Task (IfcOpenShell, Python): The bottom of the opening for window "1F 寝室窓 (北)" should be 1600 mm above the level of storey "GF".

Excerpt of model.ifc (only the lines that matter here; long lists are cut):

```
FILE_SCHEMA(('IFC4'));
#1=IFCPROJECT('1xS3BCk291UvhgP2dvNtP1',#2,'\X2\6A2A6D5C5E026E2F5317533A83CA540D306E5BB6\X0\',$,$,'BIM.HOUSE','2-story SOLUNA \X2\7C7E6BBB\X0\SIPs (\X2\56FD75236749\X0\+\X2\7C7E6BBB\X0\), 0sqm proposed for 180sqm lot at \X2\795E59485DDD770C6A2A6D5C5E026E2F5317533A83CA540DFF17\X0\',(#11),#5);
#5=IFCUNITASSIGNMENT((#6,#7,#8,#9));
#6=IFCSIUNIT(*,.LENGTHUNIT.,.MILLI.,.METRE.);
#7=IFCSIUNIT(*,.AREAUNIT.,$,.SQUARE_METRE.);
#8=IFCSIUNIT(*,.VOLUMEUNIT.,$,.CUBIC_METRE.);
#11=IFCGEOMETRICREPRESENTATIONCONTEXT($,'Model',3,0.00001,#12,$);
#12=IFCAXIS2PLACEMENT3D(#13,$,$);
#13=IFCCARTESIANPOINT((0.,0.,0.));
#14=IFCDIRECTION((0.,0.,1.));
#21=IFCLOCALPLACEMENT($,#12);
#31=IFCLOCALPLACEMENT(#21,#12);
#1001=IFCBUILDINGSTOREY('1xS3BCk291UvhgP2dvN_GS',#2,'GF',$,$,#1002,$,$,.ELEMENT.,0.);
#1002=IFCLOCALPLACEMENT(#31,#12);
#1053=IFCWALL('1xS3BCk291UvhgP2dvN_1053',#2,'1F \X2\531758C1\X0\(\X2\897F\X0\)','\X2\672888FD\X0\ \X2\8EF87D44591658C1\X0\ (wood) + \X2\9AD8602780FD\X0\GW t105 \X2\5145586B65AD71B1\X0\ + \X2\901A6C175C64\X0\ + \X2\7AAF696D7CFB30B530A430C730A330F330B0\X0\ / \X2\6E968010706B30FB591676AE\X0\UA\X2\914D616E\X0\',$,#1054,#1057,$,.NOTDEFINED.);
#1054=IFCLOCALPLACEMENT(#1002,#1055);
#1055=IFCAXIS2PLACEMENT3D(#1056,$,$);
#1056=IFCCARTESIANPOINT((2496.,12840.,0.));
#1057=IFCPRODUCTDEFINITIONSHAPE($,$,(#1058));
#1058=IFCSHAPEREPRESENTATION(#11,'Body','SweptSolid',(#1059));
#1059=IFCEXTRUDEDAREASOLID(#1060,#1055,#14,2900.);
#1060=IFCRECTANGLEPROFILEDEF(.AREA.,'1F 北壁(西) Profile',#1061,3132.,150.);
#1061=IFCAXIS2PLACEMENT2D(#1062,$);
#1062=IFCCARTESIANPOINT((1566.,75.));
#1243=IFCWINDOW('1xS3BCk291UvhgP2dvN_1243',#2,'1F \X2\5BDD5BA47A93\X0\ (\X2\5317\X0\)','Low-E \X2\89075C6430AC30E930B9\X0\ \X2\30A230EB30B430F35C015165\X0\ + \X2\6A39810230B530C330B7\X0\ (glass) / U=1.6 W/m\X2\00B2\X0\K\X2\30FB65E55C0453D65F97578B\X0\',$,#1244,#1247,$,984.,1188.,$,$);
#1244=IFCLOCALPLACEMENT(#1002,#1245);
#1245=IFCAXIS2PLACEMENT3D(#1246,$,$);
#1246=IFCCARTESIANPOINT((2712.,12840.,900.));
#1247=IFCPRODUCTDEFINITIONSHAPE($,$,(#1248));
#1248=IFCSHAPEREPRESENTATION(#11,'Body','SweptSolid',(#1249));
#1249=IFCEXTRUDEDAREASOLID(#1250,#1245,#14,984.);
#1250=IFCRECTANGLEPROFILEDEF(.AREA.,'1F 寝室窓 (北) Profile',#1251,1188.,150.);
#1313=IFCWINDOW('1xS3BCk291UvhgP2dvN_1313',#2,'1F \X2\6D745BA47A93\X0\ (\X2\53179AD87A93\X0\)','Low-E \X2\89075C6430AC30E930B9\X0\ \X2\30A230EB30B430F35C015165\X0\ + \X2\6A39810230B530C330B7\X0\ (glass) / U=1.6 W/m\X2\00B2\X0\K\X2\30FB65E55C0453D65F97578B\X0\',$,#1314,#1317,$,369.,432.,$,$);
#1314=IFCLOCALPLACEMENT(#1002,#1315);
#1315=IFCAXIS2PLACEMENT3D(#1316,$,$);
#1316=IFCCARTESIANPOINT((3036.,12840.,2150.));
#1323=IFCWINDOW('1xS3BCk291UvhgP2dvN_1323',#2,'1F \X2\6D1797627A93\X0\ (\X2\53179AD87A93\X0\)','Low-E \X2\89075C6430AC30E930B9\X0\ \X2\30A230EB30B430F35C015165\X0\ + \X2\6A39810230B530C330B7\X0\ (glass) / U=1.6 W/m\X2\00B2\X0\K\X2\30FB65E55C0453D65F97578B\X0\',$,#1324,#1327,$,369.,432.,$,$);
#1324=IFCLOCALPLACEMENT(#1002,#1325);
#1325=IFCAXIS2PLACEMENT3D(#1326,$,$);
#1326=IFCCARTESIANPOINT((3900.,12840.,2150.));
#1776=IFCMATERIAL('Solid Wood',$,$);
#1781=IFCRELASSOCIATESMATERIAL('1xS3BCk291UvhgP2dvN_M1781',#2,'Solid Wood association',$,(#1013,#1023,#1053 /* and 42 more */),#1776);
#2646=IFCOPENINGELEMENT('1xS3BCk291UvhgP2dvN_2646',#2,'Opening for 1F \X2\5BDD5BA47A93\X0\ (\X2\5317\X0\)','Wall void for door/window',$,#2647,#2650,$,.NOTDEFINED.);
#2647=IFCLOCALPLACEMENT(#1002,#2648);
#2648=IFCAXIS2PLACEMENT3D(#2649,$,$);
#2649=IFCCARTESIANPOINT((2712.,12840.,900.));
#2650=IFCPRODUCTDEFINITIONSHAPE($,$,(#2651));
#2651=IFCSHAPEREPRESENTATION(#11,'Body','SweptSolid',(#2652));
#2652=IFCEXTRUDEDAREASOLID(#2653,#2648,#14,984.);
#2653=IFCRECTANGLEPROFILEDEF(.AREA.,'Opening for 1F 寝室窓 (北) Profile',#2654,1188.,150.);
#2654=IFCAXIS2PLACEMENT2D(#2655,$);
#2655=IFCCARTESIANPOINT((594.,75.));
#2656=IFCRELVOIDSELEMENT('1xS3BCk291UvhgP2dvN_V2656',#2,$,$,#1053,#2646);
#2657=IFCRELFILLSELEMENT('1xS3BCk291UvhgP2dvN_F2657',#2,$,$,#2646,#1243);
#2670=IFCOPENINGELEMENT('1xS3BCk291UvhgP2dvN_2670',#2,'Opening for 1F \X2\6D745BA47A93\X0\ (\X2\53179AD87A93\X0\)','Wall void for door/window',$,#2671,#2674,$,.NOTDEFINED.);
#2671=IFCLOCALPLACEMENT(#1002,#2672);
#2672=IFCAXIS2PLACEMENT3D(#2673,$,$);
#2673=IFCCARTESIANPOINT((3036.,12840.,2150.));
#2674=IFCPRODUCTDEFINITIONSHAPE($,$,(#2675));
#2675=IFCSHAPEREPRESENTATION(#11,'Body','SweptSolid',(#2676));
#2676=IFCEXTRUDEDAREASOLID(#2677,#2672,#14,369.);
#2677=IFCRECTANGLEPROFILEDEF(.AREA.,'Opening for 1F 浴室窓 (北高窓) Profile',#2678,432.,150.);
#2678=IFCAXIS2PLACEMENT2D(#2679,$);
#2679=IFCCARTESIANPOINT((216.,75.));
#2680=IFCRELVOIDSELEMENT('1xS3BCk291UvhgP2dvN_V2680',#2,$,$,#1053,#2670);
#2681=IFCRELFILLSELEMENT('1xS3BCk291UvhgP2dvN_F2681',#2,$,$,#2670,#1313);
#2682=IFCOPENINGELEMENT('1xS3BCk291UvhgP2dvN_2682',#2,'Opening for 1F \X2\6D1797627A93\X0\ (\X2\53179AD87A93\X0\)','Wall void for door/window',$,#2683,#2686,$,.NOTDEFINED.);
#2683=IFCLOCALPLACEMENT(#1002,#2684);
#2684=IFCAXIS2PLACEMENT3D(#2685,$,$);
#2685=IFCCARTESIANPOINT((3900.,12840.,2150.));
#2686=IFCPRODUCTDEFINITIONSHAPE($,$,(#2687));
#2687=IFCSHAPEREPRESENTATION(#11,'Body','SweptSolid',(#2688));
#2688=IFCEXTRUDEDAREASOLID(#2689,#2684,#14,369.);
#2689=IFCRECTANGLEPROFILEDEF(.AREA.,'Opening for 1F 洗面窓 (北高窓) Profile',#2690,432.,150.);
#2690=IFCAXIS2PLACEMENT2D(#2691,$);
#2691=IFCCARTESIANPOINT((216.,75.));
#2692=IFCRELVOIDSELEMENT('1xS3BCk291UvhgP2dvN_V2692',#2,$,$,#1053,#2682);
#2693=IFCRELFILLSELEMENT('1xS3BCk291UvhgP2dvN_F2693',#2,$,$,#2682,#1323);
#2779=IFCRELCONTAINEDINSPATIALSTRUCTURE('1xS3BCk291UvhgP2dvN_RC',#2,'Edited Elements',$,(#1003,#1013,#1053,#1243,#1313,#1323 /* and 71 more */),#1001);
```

```python
import numpy as np
import ifcopenshell
import ifcopenshell.api.geometry
import ifcopenshell.geom
import ifcopenshell.util.element
import ifcopenshell.util.placement
import ifcopenshell.util.shape
import ifcopenshell.util.unit

model = ifcopenshell.open("model.ifc")
unit_scale = ifcopenshell.util.unit.calculate_unit_scale(model)

window = model.by_guid("1xS3BCk291UvhgP2dvN_1243")
opening = window.FillsVoids[0].RelatingOpeningElement
storey = ifcopenshell.util.element.get_container(window, ifc_class="IfcBuildingStorey")
level = ifcopenshell.util.placement.get_local_placement(storey.ObjectPlacement)[2, 3]

# The opening's origin need not be at the sill, so measure its lowest point.
shape = ifcopenshell.geom.create_shape(ifcopenshell.geom.settings(), opening)
bottom = ifcopenshell.util.shape.get_shape_bottom_elevation(shape, shape.geometry) / unit_scale
dz = level + 1600.0 - bottom

shift = np.array([0.0, 0.0, dz])
# The window is not placed relative to its opening, so move both.
for product in (opening, window):
    matrix = ifcopenshell.util.placement.get_local_placement(product.ObjectPlacement)
    matrix[:3, 3] += shift
    ifcopenshell.api.geometry.edit_object_placement(model, product=product, matrix=matrix, is_si=False)

print(f"moved by {dz * unit_scale:+.3f} m")

model.write("model_rev.ifc")
```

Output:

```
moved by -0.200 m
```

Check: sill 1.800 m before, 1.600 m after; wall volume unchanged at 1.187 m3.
